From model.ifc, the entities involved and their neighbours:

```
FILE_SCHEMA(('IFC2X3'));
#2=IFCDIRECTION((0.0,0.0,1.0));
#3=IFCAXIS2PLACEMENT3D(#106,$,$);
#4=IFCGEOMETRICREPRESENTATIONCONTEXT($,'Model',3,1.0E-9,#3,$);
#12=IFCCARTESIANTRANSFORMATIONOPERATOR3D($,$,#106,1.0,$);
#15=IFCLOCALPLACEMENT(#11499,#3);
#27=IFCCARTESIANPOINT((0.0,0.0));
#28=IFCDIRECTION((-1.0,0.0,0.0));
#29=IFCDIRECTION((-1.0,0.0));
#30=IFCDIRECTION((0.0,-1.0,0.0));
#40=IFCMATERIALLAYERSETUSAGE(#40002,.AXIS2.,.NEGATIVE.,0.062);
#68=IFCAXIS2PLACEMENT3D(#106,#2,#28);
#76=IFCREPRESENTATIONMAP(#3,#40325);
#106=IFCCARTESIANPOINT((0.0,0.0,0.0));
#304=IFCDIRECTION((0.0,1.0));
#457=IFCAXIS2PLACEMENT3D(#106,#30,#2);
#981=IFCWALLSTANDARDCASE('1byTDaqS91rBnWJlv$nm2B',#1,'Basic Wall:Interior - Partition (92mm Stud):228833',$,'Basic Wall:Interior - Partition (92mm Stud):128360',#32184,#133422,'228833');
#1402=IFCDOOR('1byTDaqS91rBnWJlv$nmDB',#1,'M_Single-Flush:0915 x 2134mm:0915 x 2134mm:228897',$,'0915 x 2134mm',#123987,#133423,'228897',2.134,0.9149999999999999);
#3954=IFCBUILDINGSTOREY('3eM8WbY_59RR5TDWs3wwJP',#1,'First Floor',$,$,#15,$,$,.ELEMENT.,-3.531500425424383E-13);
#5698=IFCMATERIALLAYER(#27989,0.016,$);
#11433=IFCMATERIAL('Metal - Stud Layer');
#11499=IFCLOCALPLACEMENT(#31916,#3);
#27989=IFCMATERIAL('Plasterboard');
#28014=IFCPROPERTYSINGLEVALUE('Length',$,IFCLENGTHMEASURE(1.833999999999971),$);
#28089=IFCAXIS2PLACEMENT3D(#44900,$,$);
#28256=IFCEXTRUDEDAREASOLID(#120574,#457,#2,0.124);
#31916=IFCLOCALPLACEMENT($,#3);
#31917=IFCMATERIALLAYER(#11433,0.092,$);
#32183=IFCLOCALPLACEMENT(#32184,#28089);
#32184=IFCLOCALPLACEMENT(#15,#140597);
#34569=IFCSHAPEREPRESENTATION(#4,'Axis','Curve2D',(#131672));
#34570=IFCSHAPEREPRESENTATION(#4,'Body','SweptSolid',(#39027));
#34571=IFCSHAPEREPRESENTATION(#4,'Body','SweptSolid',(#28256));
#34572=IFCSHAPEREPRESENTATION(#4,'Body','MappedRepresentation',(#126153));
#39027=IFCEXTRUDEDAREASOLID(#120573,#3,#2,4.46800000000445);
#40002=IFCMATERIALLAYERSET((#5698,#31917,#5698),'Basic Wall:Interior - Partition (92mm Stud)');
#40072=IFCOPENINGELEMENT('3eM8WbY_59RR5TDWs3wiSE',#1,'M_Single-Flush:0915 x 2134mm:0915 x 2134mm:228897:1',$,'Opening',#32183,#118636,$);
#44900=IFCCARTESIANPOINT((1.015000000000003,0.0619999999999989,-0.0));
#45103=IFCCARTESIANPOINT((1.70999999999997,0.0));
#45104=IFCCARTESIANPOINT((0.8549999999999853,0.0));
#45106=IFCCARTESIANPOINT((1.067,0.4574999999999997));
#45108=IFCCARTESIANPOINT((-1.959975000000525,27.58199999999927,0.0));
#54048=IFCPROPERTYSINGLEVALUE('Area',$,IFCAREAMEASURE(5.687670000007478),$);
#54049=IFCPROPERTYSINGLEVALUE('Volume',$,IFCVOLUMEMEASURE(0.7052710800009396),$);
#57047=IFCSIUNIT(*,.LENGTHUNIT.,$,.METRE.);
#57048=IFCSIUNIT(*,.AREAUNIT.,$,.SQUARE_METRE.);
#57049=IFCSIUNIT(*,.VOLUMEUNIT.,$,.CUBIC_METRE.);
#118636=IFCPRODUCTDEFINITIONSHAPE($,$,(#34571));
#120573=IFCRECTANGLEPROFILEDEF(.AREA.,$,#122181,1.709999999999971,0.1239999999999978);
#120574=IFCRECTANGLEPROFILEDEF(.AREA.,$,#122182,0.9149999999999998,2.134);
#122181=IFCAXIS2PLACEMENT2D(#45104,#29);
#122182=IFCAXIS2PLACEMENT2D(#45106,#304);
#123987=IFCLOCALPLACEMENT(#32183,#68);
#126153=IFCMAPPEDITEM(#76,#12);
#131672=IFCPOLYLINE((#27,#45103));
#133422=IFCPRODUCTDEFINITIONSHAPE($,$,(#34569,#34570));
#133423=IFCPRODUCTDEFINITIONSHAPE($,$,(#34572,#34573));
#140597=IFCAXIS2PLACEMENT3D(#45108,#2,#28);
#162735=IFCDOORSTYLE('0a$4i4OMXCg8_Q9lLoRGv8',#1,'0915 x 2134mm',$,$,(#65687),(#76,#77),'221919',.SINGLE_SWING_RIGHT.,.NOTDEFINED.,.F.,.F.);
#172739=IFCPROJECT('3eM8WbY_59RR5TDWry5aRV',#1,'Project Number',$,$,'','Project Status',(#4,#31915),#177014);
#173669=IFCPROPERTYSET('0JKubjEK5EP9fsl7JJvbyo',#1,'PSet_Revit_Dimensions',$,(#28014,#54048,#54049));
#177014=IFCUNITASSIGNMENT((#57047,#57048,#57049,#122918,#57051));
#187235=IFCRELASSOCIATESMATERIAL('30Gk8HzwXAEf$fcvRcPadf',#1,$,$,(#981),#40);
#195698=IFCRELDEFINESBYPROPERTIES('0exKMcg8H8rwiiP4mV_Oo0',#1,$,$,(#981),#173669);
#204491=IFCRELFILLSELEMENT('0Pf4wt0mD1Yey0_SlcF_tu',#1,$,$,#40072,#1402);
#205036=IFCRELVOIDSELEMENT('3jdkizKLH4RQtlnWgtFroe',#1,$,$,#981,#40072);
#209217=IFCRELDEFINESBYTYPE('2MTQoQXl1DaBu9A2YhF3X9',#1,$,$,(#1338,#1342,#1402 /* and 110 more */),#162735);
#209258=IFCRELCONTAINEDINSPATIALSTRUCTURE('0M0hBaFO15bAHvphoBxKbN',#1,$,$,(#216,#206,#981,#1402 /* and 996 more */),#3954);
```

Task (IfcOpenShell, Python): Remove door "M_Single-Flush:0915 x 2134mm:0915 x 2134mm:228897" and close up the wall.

```python
import ifcopenshell
import ifcopenshell.api.feature
import ifcopenshell.api.pset
import ifcopenshell.api.root
import ifcopenshell.geom
import ifcopenshell.util.element
import ifcopenshell.util.shape
import ifcopenshell.util.unit

model = ifcopenshell.open("model.ifc")
area_scale = ifcopenshell.util.unit.calculate_unit_scale(model, "AREAUNIT")
volume_scale = ifcopenshell.util.unit.calculate_unit_scale(model, "VOLUMEUNIT")
settings = ifcopenshell.geom.settings()


def volume(element):
    """Net volume in cubic metres, openings subtracted."""
    shape = ifcopenshell.geom.create_shape(settings, element)
    return ifcopenshell.util.shape.get_volume(shape.geometry)


door = model.by_guid("1byTDaqS91rBnWJlv$nmDB")
opening = door.FillsVoids[0].RelatingOpeningElement
wall = opening.VoidsElements[0].RelatingBuildingElement
before = volume(wall)

ifcopenshell.api.root.remove_product(model, product=door)
ifcopenshell.api.feature.remove_feature(model, feature=opening)

after = volume(wall)
thickness = 0.124  # wall thickness in metres

# Update the wall's stored quantities.
pset = model.by_id(ifcopenshell.util.element.get_pset(wall, "PSet_Revit_Dimensions", should_inherit=False)["id"])
ifcopenshell.api.pset.edit_pset(model, pset=pset, properties={
    "Area": model.create_entity("IfcAreaMeasure", after / thickness / area_scale),
    "Volume": model.create_entity("IfcVolumeMeasure", after / volume_scale),
})

print(f"wall volume {before:.3f} -> {after:.3f} m3")

model.write("model_rev.ifc")
```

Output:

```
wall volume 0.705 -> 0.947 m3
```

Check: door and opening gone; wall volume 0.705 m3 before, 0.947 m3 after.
